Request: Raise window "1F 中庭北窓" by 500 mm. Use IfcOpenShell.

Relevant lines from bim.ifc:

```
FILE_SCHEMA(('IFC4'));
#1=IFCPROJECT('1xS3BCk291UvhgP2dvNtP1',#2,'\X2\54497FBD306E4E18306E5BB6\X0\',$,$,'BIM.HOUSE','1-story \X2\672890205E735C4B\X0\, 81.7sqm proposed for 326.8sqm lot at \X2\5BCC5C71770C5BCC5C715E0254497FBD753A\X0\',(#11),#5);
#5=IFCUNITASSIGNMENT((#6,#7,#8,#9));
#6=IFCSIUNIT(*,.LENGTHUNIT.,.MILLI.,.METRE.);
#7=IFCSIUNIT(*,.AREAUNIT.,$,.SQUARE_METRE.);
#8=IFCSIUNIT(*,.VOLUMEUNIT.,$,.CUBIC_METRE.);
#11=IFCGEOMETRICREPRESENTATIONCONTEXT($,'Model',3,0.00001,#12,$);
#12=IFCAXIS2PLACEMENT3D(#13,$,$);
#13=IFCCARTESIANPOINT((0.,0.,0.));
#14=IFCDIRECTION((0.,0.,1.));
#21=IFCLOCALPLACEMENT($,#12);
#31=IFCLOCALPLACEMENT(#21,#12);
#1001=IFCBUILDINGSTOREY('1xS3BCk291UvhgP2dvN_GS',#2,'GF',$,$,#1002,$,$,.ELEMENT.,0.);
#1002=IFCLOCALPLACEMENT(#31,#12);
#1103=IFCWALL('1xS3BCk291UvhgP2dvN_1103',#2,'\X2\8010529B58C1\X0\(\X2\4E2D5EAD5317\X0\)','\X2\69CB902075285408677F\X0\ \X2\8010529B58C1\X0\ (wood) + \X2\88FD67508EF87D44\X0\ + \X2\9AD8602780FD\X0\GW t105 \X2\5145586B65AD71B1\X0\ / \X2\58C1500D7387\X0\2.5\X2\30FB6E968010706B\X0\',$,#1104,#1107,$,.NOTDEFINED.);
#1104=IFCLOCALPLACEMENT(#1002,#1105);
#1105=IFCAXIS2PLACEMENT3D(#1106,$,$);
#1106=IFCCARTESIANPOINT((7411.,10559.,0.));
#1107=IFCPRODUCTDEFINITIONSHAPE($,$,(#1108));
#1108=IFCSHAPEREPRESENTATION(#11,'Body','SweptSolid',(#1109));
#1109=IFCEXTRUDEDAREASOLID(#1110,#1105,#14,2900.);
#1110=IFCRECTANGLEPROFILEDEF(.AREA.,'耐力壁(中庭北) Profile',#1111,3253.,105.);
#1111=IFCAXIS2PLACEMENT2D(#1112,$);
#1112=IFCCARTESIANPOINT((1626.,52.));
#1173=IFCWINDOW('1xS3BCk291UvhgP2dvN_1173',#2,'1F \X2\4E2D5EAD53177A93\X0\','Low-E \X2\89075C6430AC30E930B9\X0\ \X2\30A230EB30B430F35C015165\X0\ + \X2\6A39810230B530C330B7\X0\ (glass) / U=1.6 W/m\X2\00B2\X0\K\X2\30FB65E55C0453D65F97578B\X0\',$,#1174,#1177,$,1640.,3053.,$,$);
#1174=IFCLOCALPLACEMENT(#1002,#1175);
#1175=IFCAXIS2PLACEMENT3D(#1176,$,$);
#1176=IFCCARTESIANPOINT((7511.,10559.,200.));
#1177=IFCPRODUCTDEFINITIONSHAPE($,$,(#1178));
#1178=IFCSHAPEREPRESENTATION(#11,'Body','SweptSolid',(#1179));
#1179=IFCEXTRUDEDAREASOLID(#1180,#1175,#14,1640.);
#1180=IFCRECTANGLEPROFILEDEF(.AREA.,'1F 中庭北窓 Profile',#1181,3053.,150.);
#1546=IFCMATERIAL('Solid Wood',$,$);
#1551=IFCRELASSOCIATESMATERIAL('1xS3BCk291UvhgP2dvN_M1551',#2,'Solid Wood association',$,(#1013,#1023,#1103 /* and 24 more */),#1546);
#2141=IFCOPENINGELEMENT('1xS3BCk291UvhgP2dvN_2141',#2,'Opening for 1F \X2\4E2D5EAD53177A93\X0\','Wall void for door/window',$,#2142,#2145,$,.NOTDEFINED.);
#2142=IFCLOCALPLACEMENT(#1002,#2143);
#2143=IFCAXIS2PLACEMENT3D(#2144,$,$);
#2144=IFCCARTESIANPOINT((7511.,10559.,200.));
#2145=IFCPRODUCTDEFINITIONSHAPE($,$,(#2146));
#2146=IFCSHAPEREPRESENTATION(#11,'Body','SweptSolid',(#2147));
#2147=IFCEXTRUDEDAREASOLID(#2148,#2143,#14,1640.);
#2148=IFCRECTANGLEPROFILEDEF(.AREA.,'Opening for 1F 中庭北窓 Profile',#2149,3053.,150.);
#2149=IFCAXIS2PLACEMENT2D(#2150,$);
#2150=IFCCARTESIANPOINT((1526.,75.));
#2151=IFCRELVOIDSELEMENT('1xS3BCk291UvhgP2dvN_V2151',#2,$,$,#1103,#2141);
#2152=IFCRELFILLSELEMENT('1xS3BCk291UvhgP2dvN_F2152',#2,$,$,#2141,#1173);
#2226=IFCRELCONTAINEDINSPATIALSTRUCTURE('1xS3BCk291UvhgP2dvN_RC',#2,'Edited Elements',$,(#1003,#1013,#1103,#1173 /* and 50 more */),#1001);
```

```python
import numpy as np
import ifcopenshell
import ifcopenshell.api.geometry
import ifcopenshell.util.placement
import ifcopenshell.util.unit

model = ifcopenshell.open("bim.ifc")
unit_scale = ifcopenshell.util.unit.calculate_unit_scale(model)

window = model.by_id(1173)
opening = window.FillsVoids[0].RelatingOpeningElement
dz = 0.5 / unit_scale

shift = np.array([0.0, 0.0, dz])
# The window is not placed relative to its opening, so move both.
for product in (opening, window):
    matrix = ifcopenshell.util.placement.get_local_placement(product.ObjectPlacement)
    matrix[:3, 3] += shift
    ifcopenshell.api.geometry.edit_object_placement(model, product=product, matrix=matrix, is_si=False)

print(f"moved by {dz * unit_scale:+.3f} m")

model.write("bim_edited.ifc")
```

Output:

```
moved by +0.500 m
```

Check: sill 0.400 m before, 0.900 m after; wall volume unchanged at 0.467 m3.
